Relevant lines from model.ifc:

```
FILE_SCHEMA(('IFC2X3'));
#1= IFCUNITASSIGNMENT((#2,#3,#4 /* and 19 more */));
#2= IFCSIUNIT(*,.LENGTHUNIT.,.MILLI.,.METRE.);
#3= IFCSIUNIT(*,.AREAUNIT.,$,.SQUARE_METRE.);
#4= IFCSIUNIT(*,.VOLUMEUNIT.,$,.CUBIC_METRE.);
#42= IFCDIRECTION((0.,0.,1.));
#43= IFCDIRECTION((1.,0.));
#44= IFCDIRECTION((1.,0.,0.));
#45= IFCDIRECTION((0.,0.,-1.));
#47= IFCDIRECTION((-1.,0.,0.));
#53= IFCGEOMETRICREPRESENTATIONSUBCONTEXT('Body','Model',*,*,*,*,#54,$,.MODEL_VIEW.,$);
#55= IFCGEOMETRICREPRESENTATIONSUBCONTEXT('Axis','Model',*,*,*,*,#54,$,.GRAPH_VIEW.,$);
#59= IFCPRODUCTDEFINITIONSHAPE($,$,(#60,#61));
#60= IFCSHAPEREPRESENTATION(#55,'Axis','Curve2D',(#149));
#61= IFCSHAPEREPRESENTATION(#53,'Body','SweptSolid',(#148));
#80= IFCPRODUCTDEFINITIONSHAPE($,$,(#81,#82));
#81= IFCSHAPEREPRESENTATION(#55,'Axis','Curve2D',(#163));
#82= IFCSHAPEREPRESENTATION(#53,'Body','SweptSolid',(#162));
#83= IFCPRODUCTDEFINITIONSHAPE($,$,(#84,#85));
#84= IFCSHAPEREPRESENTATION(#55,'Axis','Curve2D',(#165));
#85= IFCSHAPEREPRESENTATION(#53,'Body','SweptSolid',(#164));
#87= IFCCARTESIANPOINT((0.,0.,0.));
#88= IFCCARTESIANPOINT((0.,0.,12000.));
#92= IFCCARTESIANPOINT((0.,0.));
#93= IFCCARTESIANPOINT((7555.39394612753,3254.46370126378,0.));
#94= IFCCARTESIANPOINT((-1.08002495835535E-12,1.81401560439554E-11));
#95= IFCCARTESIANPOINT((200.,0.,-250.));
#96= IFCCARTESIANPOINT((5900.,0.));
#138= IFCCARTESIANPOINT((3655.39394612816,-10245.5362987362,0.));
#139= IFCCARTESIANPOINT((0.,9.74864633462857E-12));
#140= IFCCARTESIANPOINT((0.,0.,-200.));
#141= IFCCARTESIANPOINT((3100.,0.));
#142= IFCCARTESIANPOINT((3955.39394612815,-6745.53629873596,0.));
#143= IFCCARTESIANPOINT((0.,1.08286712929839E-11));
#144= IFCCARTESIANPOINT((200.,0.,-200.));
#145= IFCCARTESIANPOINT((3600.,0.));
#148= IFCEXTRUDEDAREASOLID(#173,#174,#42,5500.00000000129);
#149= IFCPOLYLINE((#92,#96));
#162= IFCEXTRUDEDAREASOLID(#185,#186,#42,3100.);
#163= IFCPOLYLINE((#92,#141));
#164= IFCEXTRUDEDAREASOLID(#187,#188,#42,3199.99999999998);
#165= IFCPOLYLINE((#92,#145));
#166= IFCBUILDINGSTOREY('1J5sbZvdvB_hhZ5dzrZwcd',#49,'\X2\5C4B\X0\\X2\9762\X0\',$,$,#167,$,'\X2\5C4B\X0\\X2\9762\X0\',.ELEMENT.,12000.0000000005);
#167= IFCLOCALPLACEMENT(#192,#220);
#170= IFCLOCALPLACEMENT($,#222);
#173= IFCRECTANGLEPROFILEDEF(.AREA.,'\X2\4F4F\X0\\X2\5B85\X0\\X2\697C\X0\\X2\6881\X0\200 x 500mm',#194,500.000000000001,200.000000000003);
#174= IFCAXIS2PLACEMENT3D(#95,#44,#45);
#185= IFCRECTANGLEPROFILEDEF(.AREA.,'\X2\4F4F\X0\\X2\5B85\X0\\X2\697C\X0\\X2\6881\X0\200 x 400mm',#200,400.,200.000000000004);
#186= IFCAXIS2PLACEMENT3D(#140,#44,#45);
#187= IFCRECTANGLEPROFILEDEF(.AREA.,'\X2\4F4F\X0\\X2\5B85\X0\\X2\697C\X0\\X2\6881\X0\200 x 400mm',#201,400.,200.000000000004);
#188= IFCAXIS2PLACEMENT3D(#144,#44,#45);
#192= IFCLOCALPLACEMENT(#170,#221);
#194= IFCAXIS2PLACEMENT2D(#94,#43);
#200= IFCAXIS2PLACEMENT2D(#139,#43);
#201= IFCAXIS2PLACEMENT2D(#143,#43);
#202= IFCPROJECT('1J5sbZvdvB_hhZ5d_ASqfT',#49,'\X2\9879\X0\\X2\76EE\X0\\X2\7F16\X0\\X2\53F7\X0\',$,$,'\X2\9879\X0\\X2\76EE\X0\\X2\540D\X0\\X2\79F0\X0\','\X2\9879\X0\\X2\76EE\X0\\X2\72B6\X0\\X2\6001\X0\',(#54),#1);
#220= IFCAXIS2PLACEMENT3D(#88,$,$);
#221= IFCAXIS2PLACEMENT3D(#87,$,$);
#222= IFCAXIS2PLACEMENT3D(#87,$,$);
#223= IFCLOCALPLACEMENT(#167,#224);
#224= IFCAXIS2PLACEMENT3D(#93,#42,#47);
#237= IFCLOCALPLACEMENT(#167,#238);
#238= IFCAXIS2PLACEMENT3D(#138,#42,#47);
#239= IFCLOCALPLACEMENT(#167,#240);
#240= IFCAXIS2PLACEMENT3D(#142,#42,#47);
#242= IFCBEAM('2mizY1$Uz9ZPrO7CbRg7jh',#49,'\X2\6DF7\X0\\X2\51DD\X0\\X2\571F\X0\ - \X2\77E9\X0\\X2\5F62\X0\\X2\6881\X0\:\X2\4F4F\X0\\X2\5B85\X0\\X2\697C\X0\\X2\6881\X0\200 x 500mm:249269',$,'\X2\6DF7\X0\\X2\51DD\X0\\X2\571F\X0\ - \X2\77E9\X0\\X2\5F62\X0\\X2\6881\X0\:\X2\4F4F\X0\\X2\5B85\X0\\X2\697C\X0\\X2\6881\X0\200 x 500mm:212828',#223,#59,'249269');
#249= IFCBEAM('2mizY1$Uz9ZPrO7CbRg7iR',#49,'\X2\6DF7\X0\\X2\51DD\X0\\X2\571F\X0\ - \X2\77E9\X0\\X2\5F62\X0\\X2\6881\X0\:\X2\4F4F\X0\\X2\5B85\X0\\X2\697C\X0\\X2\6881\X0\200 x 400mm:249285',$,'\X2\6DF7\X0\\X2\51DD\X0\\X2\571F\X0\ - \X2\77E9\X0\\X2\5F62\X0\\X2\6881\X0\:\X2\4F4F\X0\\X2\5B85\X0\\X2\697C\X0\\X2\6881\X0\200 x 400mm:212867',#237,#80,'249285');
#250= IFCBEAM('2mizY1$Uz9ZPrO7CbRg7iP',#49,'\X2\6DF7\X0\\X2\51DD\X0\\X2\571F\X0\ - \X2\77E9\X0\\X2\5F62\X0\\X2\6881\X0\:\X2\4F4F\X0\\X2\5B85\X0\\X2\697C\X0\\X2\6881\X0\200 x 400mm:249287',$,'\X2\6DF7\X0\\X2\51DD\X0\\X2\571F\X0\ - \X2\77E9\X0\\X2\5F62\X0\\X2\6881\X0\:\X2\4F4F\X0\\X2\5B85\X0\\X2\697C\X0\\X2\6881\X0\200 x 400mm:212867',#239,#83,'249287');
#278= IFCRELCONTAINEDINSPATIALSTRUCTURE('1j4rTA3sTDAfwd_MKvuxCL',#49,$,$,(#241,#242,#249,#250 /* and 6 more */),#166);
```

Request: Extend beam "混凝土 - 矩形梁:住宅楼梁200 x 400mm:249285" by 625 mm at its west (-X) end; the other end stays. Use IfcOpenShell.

```python
import numpy as np
import ifcopenshell
import ifcopenshell.util.representation
import ifcopenshell.util.unit

model = ifcopenshell.open("model.ifc")
unit_scale = ifcopenshell.util.unit.calculate_unit_scale(model)

member = model.by_guid("2mizY1$Uz9ZPrO7CbRg7iR")
change = 0.625 / unit_scale

# The extrusion runs towards the end named, so only its depth changes.
body = ifcopenshell.util.representation.get_representation(member, "Model", "Body")
solid = body.Items[0]
old_length = solid.Depth
solid.Depth += change

# Move the axis end point with it.
axis = next(r for r in member.Representation.Representations if r.RepresentationIdentifier == "Axis").Items[0]
start, end = (np.array(p.Coordinates) for p in axis.Points)
end = end + (end - start) / np.linalg.norm(end - start) * change
point = model.createIfcCartesianPoint(end.tolist())
axis.Points = [axis.Points[0], point]

print(f"length {old_length:g} -> {solid.Depth:g}")

model.write("model_v2.ifc")
```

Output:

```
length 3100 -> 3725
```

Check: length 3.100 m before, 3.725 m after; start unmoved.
